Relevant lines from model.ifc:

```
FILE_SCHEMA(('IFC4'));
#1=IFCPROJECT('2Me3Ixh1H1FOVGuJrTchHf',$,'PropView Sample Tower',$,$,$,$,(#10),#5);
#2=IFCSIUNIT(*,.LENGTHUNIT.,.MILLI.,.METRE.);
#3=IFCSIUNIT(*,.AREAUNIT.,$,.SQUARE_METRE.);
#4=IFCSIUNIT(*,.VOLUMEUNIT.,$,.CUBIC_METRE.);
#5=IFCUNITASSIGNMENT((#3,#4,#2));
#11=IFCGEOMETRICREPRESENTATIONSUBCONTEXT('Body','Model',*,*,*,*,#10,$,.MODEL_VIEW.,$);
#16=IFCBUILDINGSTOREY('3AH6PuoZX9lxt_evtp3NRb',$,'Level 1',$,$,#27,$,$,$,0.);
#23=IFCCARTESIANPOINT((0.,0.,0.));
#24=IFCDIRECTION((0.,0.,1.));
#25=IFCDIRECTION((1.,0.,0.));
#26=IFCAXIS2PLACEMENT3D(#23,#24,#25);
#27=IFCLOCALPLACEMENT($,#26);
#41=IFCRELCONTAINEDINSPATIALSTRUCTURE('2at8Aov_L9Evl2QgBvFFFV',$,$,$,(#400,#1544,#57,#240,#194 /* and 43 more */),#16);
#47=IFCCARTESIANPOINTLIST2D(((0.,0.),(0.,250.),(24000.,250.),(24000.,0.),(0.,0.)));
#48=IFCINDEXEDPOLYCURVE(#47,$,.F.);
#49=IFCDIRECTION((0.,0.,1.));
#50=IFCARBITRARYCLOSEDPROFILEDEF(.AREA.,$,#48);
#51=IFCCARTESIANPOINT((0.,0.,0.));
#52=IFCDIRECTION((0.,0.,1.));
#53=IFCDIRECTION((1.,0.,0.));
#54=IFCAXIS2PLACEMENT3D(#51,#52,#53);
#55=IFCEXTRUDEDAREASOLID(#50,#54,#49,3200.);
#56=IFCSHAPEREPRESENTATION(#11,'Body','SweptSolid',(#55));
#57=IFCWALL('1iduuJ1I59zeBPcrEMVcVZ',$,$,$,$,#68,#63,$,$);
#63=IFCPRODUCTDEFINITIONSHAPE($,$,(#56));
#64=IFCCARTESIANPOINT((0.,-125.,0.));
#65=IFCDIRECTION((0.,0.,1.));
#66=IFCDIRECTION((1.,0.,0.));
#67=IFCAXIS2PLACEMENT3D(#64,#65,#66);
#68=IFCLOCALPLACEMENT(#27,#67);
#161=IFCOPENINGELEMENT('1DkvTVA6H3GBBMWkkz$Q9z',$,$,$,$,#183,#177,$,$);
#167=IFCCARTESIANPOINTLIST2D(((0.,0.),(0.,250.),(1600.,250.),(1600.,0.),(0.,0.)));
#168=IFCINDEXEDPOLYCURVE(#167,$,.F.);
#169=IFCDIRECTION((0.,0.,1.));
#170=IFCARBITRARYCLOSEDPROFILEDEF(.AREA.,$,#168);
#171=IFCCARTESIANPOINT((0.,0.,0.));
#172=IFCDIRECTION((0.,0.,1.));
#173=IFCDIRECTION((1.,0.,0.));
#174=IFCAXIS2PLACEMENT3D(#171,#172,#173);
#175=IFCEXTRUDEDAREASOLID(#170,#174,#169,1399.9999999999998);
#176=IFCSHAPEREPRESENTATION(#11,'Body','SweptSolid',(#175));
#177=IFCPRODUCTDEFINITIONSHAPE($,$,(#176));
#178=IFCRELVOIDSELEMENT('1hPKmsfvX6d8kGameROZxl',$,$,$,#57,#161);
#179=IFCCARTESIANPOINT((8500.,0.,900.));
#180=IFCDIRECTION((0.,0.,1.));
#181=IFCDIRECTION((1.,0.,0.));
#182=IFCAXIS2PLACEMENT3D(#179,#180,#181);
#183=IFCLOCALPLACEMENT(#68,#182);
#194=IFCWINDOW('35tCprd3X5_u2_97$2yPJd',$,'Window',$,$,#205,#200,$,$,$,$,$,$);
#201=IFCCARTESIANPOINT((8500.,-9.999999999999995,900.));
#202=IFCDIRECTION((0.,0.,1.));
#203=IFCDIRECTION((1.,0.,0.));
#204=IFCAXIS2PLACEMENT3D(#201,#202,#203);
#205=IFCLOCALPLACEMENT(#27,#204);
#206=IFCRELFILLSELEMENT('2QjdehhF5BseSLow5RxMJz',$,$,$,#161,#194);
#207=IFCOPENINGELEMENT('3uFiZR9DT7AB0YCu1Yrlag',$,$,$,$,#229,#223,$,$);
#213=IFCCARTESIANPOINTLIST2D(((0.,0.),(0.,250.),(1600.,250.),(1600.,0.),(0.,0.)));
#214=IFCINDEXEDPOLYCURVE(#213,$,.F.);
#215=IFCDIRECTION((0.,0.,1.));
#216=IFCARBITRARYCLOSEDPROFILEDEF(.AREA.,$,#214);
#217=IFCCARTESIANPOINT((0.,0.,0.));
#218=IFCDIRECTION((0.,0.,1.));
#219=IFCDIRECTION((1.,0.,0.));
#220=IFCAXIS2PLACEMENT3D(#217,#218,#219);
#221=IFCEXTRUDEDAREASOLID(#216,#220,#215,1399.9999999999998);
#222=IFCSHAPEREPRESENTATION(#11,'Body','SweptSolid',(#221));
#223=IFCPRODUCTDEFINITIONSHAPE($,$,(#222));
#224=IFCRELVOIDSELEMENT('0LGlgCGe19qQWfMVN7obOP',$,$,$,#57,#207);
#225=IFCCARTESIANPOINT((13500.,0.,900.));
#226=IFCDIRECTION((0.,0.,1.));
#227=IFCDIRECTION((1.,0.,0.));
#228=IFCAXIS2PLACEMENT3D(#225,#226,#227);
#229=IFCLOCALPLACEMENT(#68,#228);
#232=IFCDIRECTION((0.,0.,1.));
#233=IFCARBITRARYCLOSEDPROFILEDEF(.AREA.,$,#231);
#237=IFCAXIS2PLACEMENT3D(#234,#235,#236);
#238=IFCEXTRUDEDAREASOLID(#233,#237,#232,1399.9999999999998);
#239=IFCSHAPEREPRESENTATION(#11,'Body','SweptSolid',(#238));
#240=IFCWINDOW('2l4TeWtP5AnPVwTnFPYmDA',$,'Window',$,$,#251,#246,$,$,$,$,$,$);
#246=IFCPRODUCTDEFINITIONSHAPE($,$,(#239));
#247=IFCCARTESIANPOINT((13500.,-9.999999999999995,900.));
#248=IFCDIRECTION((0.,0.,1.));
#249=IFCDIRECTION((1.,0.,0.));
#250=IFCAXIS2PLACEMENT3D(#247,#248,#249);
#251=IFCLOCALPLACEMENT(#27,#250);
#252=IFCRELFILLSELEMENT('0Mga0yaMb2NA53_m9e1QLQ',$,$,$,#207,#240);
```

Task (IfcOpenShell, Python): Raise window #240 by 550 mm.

```python
import numpy as np
import ifcopenshell
import ifcopenshell.api.geometry
import ifcopenshell.util.placement
import ifcopenshell.util.unit

model = ifcopenshell.open("model.ifc")
unit_scale = ifcopenshell.util.unit.calculate_unit_scale(model)

window = model.by_guid("2l4TeWtP5AnPVwTnFPYmDA")
opening = window.FillsVoids[0].RelatingOpeningElement
dz = 550.0

shift = np.array([0.0, 0.0, dz])
# The window is not placed relative to its opening, so move both.
for product in (opening, window):
    matrix = ifcopenshell.util.placement.get_local_placement(product.ObjectPlacement)
    matrix[:3, 3] += shift
    ifcopenshell.api.geometry.edit_object_placement(model, product=product, matrix=matrix, is_si=False)

print(f"moved by {dz * unit_scale:+.3f} m")

model.write("model_rev.ifc")
```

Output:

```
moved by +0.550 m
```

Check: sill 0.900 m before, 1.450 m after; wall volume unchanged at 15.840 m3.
